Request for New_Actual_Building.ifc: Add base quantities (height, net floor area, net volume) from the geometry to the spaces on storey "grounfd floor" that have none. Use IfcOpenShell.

First a look at what the model holds.

```python
import ifcopenshell
import ifcopenshell.util.element
import ifcopenshell.util.unit

model = ifcopenshell.open("New_Actual_Building.ifc")
print(model.schema)
for unit_type in ("LENGTHUNIT", "AREAUNIT", "VOLUMEUNIT"):
    print(unit_type, ifcopenshell.util.unit.calculate_unit_scale(model, unit_type))
storey = next(s for s in model.by_type("IfcBuildingStorey") if s.Name == "grounfd floor")
spaces = [e for e in ifcopenshell.util.element.get_decomposition(storey) if e.is_a("IfcSpace")]
for e in sorted(spaces, key=lambda e: e.id()):
    print(e.id(), e.is_a(), e.Name, list(ifcopenshell.util.element.get_psets(e, qtos_only=True)), sep=" | ")
```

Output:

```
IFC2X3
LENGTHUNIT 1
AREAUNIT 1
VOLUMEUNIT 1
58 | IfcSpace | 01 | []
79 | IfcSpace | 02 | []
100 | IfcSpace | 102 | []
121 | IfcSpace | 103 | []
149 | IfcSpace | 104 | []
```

```python
import ifcopenshell
import ifcopenshell.api.pset
import ifcopenshell.geom
import ifcopenshell.util.element
import ifcopenshell.util.shape
import ifcopenshell.util.unit

model = ifcopenshell.open("New_Actual_Building.ifc")
unit_scale = ifcopenshell.util.unit.calculate_unit_scale(model)
area_scale = ifcopenshell.util.unit.calculate_unit_scale(model, "AREAUNIT")
volume_scale = ifcopenshell.util.unit.calculate_unit_scale(model, "VOLUMEUNIT")
settings = ifcopenshell.geom.settings()

storey = next(s for s in model.by_type("IfcBuildingStorey") if s.Name == "grounfd floor")
spaces = [e for e in ifcopenshell.util.element.get_decomposition(storey) if e.is_a("IfcSpace")]

for e in sorted(spaces, key=lambda e: e.id()):
    if ifcopenshell.util.element.get_psets(e, qtos_only=True, should_inherit=False):
        continue
    # Geometry comes back in metres, in the element's own axes.
    shape = ifcopenshell.geom.create_shape(settings, e)
    values = {
        "Height": ifcopenshell.util.shape.get_z(shape.geometry) / unit_scale,
        "NetFloorArea": ifcopenshell.util.shape.get_footprint_area(shape.geometry) / area_scale,
        "NetVolume": ifcopenshell.util.shape.get_volume(shape.geometry) / volume_scale,
    }
    qto = ifcopenshell.api.pset.add_qto(model, product=e, name="BaseQuantities")
    ifcopenshell.api.pset.edit_qto(model, qto=qto, properties=values)
    print(e.id(), {k: round(v, 3) for k, v in values.items()})

model.write("New_Actual_Building-out.ifc")
```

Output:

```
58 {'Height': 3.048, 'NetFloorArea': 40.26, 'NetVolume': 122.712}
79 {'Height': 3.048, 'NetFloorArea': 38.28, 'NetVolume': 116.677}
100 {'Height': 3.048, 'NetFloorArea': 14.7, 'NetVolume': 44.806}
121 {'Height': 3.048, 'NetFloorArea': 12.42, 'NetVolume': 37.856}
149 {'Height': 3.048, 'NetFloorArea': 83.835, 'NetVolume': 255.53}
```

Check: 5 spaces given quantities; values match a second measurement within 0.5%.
